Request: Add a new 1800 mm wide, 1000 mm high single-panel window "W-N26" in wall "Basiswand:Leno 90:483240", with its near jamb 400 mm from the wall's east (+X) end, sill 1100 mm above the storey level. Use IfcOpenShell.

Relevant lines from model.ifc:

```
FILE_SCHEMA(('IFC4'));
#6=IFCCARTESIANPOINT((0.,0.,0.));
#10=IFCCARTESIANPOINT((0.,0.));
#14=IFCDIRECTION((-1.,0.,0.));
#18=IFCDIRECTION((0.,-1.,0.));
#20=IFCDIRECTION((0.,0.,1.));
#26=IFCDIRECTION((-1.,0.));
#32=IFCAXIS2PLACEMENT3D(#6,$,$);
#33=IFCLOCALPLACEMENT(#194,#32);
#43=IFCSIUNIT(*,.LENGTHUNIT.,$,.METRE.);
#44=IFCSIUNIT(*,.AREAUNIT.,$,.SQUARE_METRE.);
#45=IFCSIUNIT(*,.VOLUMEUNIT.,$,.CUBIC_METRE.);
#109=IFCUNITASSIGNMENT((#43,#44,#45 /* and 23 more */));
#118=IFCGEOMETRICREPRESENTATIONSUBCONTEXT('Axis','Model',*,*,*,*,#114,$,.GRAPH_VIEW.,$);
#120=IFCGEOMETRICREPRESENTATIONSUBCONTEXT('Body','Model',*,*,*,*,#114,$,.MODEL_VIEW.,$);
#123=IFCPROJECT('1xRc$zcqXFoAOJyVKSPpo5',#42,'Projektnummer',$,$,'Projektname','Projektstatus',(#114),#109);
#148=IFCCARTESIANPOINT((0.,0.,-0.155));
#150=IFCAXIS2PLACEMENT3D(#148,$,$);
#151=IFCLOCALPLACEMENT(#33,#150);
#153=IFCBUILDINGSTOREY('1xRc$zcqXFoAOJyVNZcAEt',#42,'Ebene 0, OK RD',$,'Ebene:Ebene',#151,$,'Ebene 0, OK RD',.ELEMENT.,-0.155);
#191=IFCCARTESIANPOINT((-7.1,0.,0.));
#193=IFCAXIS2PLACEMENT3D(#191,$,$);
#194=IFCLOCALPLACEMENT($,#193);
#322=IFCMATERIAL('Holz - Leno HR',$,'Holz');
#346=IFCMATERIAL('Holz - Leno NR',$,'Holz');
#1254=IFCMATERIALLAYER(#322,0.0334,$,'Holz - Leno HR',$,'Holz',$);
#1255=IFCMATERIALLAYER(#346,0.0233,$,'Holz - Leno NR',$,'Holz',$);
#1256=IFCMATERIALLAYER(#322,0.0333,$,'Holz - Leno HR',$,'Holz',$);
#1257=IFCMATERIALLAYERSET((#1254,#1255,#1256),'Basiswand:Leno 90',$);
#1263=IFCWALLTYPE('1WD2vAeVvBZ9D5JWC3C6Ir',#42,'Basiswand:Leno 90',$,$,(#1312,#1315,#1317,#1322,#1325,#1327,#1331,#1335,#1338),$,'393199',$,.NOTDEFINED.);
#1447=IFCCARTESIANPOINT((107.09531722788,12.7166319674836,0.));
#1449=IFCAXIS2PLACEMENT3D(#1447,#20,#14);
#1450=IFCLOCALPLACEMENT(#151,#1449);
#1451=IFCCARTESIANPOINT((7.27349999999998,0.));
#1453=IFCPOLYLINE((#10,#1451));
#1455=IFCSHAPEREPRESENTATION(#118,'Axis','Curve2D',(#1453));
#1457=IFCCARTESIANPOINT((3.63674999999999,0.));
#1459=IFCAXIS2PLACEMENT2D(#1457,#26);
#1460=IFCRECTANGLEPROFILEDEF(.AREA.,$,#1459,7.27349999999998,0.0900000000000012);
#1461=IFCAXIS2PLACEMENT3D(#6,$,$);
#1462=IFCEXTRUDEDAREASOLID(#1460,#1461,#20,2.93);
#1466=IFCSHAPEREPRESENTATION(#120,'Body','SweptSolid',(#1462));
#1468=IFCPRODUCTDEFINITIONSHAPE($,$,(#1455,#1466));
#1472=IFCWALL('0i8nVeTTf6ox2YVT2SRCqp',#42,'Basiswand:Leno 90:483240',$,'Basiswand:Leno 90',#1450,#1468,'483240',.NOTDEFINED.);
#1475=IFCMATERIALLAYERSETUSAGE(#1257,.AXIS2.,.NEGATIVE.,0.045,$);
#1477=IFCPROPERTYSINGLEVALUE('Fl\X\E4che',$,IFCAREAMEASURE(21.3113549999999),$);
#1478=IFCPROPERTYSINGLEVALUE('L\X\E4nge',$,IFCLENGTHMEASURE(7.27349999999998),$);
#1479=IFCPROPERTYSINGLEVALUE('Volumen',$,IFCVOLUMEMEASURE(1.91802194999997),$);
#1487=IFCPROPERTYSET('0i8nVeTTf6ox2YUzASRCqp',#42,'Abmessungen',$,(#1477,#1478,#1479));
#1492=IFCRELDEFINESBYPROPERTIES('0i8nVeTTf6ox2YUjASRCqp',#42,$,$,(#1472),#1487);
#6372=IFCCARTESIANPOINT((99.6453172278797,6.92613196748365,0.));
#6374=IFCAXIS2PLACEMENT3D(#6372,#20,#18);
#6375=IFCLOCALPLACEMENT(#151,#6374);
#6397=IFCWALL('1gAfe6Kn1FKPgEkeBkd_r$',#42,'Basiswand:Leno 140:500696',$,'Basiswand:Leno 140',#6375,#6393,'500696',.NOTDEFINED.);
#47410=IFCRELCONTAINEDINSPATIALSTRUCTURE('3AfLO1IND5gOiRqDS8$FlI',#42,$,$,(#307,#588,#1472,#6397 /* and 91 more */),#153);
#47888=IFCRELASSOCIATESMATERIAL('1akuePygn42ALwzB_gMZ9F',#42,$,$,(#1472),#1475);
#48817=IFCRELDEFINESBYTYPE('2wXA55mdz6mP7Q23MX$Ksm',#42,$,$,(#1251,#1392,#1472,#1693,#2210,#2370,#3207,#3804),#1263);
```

```python
import numpy as np
import ifcopenshell
import ifcopenshell.api.feature
import ifcopenshell.api.geometry
import ifcopenshell.api.pset
import ifcopenshell.api.root
import ifcopenshell.api.spatial
import ifcopenshell.geom
import ifcopenshell.util.element
import ifcopenshell.util.placement
import ifcopenshell.util.representation
import ifcopenshell.util.shape
import ifcopenshell.util.unit

model = ifcopenshell.open("model.ifc")
unit_scale = ifcopenshell.util.unit.calculate_unit_scale(model)
area_scale = ifcopenshell.util.unit.calculate_unit_scale(model, "AREAUNIT")
volume_scale = ifcopenshell.util.unit.calculate_unit_scale(model, "VOLUMEUNIT")
settings = ifcopenshell.geom.settings()


def volume(element):
    """Net volume in cubic metres, openings subtracted."""
    shape = ifcopenshell.geom.create_shape(settings, element)
    return ifcopenshell.util.shape.get_volume(shape.geometry)


wall = model.by_id(1472)
storey = ifcopenshell.util.element.get_container(wall, ifc_class="IfcBuildingStorey")
context = ifcopenshell.util.representation.get_context(model, "Model", "Body", "MODEL_VIEW")
before = volume(wall)

width, height, from_end, sill = 1.8, 1, 0.4, 1.1  # metres

# The wall runs along its own X axis, and the end named is its -X end.
wall_shape = ifcopenshell.geom.create_shape(settings, wall)
x, y, z = ifcopenshell.util.shape.get_vertices(wall_shape.geometry).T
start = x.min() + from_end
face, thickness = float(y.min()), float(y.max() - y.min())
wall_matrix = ifcopenshell.util.placement.get_local_placement(wall.ObjectPlacement)
level = ifcopenshell.util.placement.get_local_placement(storey.ObjectPlacement)[2, 3]


def in_wall(x, y):
    """Placement at x, y metres in the wall's axes, at sill height."""
    matrix = wall_matrix.copy()
    matrix[:, 3] = wall_matrix @ np.array([x / unit_scale, y / unit_scale, 0.0, 1.0])
    matrix[2, 3] = level + sill / unit_scale
    return matrix


# Opening: a box that overshoots both wall faces by 50 mm.
opening = ifcopenshell.api.root.create_entity(model, ifc_class="IfcOpeningElement", predefined_type="OPENING")
box = ifcopenshell.api.geometry.add_wall_representation(
    model, context=context, length=width, height=height, thickness=thickness + 0.1
)
ifcopenshell.api.geometry.assign_representation(model, product=opening, representation=box)
ifcopenshell.api.geometry.edit_object_placement(model, product=opening, matrix=in_wall(start, face - 0.05), is_si=False)
ifcopenshell.api.feature.add_feature(model, feature=opening, element=wall)

window = ifcopenshell.api.root.create_entity(model, ifc_class="IfcWindow", name="W-N26", predefined_type="WINDOW")
window.OverallWidth, window.OverallHeight = width / unit_scale, height / unit_scale
window.PartitioningType = "SINGLE_PANEL"
body = ifcopenshell.api.geometry.add_window_representation(
    model,
    context=context,
    overall_width=window.OverallWidth,
    overall_height=window.OverallHeight,
    partition_type="SINGLE_PANEL",
)
ifcopenshell.api.geometry.assign_representation(model, product=window, representation=body)
ifcopenshell.api.spatial.assign_container(model, products=[window], relating_structure=storey)
ifcopenshell.api.feature.add_filling(model, opening=opening, element=window)

# Centre the window in the wall's thickness.
ifcopenshell.api.geometry.edit_object_placement(model, product=window, matrix=in_wall(start, face), is_si=False)
window_shape = ifcopenshell.geom.create_shape(settings, window)
depth = ifcopenshell.util.shape.get_vertices(window_shape.geometry)[:, 1]
offset = face + thickness / 2 - (depth.min() + depth.max()) / 2
ifcopenshell.api.geometry.edit_object_placement(model, product=window, matrix=in_wall(start, offset), is_si=False)

after = volume(wall)

# Update the wall's stored quantities.
pset = model.by_id(ifcopenshell.util.element.get_pset(wall, "Abmessungen", should_inherit=False)["id"])
ifcopenshell.api.pset.edit_pset(model, pset=pset, properties={
    "Fläche": model.create_entity("IfcAreaMeasure", after / thickness / area_scale),
    "Volumen": model.create_entity("IfcVolumeMeasure", after / volume_scale),
})

print(f"wall volume {before:.3f} -> {after:.3f} m3")

model.write("model_updated.ifc")
```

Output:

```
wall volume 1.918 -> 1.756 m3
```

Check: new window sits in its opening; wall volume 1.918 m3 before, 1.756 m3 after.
